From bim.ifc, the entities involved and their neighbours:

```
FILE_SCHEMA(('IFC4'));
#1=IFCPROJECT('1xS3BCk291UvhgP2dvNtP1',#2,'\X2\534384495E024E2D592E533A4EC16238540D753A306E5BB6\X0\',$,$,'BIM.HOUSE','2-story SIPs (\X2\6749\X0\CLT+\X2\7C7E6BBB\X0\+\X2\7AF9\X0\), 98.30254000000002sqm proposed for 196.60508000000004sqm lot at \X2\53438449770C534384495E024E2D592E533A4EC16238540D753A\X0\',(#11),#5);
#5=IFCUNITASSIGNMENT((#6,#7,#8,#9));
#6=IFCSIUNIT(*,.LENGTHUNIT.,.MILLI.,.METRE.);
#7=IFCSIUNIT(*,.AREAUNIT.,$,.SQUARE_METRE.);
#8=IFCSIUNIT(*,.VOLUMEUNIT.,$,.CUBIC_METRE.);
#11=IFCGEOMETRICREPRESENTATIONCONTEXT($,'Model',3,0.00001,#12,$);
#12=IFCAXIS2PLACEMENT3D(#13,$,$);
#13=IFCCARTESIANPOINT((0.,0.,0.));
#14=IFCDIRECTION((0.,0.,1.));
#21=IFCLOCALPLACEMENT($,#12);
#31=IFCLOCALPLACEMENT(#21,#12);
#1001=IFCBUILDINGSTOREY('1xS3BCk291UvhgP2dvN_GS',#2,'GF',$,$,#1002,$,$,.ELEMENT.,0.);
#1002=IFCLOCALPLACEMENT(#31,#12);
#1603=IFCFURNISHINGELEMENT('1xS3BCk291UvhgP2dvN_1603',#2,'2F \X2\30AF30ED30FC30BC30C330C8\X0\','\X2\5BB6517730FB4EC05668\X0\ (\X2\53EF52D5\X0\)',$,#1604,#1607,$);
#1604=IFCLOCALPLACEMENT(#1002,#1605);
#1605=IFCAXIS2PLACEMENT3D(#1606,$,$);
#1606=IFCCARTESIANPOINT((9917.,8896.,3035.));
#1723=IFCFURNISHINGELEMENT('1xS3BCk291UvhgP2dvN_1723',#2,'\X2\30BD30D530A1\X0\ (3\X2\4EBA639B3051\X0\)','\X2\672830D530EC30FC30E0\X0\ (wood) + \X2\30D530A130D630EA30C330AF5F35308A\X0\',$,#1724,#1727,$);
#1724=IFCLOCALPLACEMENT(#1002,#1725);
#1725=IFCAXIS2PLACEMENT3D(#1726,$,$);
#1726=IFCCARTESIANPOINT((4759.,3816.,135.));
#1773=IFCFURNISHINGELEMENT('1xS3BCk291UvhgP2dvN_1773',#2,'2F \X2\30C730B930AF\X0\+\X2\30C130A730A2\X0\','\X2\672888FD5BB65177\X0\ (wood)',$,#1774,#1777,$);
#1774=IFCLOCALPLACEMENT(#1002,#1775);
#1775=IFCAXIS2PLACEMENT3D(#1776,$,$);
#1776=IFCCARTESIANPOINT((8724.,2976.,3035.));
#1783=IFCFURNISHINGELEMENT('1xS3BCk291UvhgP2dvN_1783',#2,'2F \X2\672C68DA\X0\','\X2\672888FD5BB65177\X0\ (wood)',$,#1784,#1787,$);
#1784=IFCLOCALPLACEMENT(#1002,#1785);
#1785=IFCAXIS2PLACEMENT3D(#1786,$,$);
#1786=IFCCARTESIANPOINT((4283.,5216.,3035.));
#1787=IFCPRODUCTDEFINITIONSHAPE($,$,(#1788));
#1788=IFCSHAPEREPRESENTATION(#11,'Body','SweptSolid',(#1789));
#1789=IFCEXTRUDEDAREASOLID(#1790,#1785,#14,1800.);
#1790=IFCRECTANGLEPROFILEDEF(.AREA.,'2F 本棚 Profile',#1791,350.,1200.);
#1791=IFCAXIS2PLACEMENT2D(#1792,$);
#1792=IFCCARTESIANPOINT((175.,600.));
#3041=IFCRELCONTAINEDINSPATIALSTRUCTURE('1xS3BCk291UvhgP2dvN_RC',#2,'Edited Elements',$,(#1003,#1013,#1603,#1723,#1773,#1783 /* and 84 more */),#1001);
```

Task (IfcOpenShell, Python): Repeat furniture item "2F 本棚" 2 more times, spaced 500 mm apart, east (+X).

```python
import numpy as np
import ifcopenshell
import ifcopenshell.api.geometry
import ifcopenshell.api.root
import ifcopenshell.util.element
import ifcopenshell.util.placement

model = ifcopenshell.open("bim.ifc")


def reuse_history(source, copy):
    """copy_class also copies each property set's owner history, people and application; keep the originals."""
    for rel in copy.IsDefinedBy:
        if rel.is_a("IfcRelDefinesByProperties") and (history := rel.RelatingPropertyDefinition.OwnerHistory):
            rel.RelatingPropertyDefinition.OwnerHistory = source.OwnerHistory
            ifcopenshell.util.element.remove_deep2(model, history)


source = model.by_id(1783)
base = ifcopenshell.util.placement.get_local_placement(source.ObjectPlacement)
step = np.array([1.0, 0.0, 0.0]) * 500.0

for i in range(1, 3):
    copy = ifcopenshell.api.root.copy_class(model, product=source)
    copy.Representation = ifcopenshell.util.element.copy_deep(
        model, source.Representation, exclude=["IfcGeometricRepresentationContext", "IfcRepresentationMap"]
    )
    reuse_history(source, copy)
    matrix = base.copy()
    matrix[:3, 3] += i * step
    print("added at", matrix[:3, 3].round(3) + 0.0)
    ifcopenshell.api.geometry.edit_object_placement(model, product=copy, matrix=matrix, is_si=False)

model.write("bim-out.ifc")
```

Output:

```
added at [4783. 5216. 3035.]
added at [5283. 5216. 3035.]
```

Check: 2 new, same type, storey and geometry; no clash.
